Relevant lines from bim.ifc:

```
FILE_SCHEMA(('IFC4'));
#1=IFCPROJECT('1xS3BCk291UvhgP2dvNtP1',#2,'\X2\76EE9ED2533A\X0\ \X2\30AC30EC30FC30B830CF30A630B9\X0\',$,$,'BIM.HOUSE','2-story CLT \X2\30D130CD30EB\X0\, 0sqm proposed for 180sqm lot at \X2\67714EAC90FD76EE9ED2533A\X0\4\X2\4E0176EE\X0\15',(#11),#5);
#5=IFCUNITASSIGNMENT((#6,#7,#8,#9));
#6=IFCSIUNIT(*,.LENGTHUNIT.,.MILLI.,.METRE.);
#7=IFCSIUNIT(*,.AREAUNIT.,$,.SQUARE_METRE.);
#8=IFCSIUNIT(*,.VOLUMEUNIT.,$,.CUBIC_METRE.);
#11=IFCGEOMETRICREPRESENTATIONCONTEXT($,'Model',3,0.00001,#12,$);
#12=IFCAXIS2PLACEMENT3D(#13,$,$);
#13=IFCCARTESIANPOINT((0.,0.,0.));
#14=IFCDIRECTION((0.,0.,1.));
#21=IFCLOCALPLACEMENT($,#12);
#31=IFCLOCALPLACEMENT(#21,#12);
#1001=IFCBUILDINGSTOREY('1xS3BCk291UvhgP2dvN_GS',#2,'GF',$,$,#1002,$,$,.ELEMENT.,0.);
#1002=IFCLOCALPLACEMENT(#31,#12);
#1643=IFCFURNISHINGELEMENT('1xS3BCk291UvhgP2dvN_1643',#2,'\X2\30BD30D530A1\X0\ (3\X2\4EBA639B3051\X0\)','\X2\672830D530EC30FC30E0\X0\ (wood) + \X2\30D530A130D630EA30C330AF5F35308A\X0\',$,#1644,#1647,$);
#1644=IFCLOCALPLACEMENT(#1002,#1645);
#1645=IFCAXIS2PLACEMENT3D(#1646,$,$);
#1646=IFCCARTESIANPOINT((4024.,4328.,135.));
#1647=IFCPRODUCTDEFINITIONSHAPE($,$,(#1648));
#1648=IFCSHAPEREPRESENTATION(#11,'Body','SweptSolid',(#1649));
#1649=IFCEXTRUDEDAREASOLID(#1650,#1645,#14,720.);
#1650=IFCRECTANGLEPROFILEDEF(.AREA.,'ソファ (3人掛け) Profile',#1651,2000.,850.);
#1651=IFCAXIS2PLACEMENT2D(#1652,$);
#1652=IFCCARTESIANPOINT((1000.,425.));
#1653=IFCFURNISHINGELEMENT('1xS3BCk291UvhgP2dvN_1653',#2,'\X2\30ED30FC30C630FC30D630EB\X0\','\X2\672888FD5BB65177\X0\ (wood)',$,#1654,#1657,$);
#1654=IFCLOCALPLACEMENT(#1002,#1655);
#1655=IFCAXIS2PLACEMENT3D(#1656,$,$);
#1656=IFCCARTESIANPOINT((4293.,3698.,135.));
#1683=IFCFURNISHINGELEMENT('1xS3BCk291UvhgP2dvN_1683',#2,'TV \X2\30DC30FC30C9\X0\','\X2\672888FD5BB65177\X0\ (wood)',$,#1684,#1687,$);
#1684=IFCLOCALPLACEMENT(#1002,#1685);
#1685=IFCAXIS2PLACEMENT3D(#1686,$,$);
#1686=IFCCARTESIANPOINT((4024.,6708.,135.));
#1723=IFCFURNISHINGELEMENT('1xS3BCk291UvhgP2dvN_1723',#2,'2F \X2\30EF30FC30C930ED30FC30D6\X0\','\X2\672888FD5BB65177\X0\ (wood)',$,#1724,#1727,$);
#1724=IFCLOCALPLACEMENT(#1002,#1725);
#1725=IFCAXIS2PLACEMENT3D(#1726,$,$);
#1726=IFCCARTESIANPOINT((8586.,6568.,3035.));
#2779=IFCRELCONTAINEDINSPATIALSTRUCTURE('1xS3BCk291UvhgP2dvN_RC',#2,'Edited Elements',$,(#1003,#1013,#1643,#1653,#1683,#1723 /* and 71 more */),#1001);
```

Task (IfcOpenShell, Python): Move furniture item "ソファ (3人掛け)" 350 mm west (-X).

```python
import ifcopenshell
import ifcopenshell.api.geometry
import ifcopenshell.util.placement
import ifcopenshell.util.unit

model = ifcopenshell.open("bim.ifc")
unit_scale = ifcopenshell.util.unit.calculate_unit_scale(model)

item = model.by_id(1643)
matrix = ifcopenshell.util.placement.get_local_placement(item.ObjectPlacement)
matrix[0, 3] -= 0.35 / unit_scale
ifcopenshell.api.geometry.edit_object_placement(model, product=item, matrix=matrix, is_si=False)

print(ifcopenshell.util.placement.get_local_placement(item.ObjectPlacement).round(3) + 0.0)

model.write("bim_rev.ifc")
```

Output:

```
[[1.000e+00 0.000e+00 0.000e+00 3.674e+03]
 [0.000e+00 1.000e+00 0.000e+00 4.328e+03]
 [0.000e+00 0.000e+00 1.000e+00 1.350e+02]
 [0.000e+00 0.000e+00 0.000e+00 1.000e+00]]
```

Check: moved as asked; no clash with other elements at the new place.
